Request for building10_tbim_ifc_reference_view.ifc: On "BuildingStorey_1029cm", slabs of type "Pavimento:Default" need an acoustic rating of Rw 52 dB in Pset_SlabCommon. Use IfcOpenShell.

First a look at what the model holds.

```python
import ifcopenshell
import ifcopenshell.util.element

model = ifcopenshell.open("building10_tbim_ifc_reference_view.ifc")
print(model.schema)
storey = next(s for s in model.by_type("IfcBuildingStorey") if s.Name == "BuildingStorey_1029cm")
slabs = [e for e in ifcopenshell.util.element.get_decomposition(storey) if e.is_a("IfcSlab")]
seen = {}
for e in slabs:
    element_type = ifcopenshell.util.element.get_type(e)
    key = (element_type.Name if element_type != e and element_type else None, ifcopenshell.util.element.get_pset(e, "Pset_SlabCommon", "AcousticRating"))
    seen[key] = seen.get(key, 0) + 1
for (name, value), count in sorted(seen.items(), key=str):
    print(count, "x", name, "|", value)
```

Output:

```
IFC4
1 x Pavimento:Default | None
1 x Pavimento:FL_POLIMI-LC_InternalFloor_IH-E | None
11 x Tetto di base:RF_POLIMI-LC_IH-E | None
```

```python
import ifcopenshell
import ifcopenshell.api.pset
import ifcopenshell.util.element

model = ifcopenshell.open("building10_tbim_ifc_reference_view.ifc")

storey = next(s for s in model.by_type("IfcBuildingStorey") if s.Name == "BuildingStorey_1029cm")
slabs = [e for e in ifcopenshell.util.element.get_decomposition(storey) if e.is_a("IfcSlab")]

count = 0
for e in slabs:
    element_type = ifcopenshell.util.element.get_type(e)
    if element_type in (None, e) or element_type.Name != "Pavimento:Default":
        continue
    # add_pset returns the element's existing set when there is one.
    pset = ifcopenshell.api.pset.add_pset(model, product=e, name="Pset_SlabCommon")
    ifcopenshell.api.pset.edit_pset(model, pset=pset, properties={"AcousticRating": "Rw 52 dB"})
    count += 1

print(count, "slabs updated")

model.write("building10_tbim_ifc_reference_view_updated.ifc")
```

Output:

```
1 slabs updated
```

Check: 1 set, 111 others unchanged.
